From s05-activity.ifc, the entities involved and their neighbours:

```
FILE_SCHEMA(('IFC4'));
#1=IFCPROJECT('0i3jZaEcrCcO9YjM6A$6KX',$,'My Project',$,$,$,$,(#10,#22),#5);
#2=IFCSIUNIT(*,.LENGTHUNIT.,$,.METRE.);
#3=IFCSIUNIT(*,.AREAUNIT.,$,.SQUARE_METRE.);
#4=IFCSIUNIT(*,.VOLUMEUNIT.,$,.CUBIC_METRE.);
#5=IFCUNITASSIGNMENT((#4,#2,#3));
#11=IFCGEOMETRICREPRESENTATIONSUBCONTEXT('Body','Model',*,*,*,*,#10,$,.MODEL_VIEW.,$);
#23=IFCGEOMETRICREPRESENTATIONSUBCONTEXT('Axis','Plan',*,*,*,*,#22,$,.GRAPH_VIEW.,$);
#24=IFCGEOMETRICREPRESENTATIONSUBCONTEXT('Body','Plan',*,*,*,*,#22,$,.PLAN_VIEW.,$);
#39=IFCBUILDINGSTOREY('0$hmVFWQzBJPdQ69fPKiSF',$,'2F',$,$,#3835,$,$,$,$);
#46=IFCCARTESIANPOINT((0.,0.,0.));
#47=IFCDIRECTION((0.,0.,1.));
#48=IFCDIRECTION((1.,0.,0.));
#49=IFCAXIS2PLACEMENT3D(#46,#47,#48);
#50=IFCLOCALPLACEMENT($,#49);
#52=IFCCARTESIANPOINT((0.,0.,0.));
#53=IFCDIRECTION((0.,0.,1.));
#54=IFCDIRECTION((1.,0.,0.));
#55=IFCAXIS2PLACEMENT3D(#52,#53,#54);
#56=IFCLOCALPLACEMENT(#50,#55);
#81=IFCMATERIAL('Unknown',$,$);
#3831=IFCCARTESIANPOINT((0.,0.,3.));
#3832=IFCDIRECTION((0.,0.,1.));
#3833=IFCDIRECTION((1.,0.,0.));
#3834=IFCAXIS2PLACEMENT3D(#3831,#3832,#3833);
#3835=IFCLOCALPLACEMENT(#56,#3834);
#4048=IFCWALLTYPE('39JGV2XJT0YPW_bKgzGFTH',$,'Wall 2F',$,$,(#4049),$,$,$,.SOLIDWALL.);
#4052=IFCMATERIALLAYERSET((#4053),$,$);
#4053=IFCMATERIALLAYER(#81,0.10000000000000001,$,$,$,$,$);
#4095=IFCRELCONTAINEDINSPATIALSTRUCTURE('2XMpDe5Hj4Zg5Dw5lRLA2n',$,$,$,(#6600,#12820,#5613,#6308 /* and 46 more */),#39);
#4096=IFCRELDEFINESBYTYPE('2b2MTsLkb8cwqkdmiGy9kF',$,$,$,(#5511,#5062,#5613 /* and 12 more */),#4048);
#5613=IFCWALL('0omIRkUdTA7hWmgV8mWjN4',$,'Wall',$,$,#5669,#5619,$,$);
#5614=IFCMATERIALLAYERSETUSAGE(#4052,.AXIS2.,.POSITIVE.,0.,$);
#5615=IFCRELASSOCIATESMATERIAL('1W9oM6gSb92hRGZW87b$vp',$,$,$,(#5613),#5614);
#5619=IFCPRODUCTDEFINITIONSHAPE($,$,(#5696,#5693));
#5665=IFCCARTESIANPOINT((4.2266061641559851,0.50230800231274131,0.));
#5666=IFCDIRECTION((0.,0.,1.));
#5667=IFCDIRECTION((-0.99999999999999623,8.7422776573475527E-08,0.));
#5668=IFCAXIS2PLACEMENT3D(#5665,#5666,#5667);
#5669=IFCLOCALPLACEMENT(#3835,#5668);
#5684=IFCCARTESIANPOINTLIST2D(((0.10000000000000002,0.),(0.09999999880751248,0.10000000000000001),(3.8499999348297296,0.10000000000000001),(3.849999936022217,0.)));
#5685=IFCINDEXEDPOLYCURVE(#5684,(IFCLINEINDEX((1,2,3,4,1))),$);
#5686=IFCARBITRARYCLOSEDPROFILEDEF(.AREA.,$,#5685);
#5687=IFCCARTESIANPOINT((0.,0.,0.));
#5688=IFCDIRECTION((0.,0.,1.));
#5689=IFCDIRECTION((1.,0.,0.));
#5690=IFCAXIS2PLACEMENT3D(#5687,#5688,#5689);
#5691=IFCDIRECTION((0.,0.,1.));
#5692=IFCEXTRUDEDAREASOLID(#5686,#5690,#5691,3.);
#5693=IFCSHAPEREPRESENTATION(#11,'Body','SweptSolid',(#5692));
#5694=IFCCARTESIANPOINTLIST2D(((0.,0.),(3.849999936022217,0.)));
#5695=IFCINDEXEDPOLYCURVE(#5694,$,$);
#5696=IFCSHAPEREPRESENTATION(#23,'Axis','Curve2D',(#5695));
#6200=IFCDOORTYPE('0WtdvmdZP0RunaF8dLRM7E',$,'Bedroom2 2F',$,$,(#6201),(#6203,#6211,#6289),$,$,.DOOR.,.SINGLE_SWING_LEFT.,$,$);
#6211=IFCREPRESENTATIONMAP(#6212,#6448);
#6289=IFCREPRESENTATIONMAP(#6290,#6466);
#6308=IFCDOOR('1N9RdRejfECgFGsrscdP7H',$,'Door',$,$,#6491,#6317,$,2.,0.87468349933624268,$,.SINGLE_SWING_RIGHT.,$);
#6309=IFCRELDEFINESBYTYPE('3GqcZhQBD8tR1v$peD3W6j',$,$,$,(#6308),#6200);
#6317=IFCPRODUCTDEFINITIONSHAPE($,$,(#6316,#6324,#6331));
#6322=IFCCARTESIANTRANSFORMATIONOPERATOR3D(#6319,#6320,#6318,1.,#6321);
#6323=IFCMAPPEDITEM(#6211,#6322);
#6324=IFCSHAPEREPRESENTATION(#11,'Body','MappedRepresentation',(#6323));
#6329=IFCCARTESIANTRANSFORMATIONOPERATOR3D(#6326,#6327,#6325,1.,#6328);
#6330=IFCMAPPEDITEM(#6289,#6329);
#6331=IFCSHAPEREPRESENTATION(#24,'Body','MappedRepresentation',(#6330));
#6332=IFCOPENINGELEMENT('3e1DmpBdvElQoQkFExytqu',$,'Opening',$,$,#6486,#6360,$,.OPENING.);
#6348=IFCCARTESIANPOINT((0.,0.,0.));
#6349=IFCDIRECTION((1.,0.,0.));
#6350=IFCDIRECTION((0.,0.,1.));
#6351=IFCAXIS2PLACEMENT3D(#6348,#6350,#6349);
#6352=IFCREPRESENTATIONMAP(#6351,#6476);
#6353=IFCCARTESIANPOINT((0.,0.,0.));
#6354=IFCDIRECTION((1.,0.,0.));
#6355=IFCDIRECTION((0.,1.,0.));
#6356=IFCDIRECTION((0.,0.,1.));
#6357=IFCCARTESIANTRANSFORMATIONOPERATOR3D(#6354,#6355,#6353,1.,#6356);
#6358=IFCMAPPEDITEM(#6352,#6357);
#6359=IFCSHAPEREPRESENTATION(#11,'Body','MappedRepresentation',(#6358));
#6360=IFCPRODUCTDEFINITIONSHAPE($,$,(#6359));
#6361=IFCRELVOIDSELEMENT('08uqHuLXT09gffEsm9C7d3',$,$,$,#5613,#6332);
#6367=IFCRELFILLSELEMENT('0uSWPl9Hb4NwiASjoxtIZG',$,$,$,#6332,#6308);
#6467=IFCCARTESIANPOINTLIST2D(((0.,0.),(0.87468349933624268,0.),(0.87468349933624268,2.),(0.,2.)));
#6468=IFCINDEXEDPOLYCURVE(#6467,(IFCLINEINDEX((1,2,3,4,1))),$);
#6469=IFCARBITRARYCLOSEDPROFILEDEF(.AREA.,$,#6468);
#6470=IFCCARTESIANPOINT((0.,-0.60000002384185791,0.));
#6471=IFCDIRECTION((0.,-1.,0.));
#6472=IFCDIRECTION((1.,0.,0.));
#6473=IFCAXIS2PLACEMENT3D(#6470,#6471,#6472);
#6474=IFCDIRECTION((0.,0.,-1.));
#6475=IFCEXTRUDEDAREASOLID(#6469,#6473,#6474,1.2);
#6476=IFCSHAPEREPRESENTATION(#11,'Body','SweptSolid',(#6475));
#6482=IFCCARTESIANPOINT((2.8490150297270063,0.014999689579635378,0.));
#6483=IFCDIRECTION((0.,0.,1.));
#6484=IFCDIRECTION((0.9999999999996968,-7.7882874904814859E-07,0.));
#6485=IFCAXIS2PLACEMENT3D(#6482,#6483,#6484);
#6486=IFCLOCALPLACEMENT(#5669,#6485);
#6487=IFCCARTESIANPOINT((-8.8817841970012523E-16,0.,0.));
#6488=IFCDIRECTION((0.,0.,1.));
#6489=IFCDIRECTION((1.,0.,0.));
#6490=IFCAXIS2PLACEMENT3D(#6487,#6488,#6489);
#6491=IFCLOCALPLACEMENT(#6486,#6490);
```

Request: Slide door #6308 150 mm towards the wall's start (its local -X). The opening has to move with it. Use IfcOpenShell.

```python
import ifcopenshell
import ifcopenshell.api.geometry
import ifcopenshell.util.placement
import ifcopenshell.util.unit

model = ifcopenshell.open("s05-activity.ifc")
unit_scale = ifcopenshell.util.unit.calculate_unit_scale(model)

door = model.by_guid("1N9RdRejfECgFGsrscdP7H")
opening = door.FillsVoids[0].RelatingOpeningElement
wall = opening.VoidsElements[0].RelatingBuildingElement

wall_matrix = ifcopenshell.util.placement.get_local_placement(wall.ObjectPlacement)
shift = wall_matrix[:3, 0] * -0.15 / unit_scale
before = ifcopenshell.util.placement.get_local_placement(door.ObjectPlacement)[:3, 3].copy()

# The door is placed relative to its opening, so it follows when the opening moves.
matrix = ifcopenshell.util.placement.get_local_placement(opening.ObjectPlacement)
matrix[:3, 3] += shift
ifcopenshell.api.geometry.edit_object_placement(
    model, product=opening, matrix=matrix, is_si=False, should_transform_children=True
)

after = ifcopenshell.util.placement.get_local_placement(door.ObjectPlacement)[:3, 3]
print("door moved by", (after - before).round(3) + 0.0)

model.write("s05-activity_rev.ifc")
```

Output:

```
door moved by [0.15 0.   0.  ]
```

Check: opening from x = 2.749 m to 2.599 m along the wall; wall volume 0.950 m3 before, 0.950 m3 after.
